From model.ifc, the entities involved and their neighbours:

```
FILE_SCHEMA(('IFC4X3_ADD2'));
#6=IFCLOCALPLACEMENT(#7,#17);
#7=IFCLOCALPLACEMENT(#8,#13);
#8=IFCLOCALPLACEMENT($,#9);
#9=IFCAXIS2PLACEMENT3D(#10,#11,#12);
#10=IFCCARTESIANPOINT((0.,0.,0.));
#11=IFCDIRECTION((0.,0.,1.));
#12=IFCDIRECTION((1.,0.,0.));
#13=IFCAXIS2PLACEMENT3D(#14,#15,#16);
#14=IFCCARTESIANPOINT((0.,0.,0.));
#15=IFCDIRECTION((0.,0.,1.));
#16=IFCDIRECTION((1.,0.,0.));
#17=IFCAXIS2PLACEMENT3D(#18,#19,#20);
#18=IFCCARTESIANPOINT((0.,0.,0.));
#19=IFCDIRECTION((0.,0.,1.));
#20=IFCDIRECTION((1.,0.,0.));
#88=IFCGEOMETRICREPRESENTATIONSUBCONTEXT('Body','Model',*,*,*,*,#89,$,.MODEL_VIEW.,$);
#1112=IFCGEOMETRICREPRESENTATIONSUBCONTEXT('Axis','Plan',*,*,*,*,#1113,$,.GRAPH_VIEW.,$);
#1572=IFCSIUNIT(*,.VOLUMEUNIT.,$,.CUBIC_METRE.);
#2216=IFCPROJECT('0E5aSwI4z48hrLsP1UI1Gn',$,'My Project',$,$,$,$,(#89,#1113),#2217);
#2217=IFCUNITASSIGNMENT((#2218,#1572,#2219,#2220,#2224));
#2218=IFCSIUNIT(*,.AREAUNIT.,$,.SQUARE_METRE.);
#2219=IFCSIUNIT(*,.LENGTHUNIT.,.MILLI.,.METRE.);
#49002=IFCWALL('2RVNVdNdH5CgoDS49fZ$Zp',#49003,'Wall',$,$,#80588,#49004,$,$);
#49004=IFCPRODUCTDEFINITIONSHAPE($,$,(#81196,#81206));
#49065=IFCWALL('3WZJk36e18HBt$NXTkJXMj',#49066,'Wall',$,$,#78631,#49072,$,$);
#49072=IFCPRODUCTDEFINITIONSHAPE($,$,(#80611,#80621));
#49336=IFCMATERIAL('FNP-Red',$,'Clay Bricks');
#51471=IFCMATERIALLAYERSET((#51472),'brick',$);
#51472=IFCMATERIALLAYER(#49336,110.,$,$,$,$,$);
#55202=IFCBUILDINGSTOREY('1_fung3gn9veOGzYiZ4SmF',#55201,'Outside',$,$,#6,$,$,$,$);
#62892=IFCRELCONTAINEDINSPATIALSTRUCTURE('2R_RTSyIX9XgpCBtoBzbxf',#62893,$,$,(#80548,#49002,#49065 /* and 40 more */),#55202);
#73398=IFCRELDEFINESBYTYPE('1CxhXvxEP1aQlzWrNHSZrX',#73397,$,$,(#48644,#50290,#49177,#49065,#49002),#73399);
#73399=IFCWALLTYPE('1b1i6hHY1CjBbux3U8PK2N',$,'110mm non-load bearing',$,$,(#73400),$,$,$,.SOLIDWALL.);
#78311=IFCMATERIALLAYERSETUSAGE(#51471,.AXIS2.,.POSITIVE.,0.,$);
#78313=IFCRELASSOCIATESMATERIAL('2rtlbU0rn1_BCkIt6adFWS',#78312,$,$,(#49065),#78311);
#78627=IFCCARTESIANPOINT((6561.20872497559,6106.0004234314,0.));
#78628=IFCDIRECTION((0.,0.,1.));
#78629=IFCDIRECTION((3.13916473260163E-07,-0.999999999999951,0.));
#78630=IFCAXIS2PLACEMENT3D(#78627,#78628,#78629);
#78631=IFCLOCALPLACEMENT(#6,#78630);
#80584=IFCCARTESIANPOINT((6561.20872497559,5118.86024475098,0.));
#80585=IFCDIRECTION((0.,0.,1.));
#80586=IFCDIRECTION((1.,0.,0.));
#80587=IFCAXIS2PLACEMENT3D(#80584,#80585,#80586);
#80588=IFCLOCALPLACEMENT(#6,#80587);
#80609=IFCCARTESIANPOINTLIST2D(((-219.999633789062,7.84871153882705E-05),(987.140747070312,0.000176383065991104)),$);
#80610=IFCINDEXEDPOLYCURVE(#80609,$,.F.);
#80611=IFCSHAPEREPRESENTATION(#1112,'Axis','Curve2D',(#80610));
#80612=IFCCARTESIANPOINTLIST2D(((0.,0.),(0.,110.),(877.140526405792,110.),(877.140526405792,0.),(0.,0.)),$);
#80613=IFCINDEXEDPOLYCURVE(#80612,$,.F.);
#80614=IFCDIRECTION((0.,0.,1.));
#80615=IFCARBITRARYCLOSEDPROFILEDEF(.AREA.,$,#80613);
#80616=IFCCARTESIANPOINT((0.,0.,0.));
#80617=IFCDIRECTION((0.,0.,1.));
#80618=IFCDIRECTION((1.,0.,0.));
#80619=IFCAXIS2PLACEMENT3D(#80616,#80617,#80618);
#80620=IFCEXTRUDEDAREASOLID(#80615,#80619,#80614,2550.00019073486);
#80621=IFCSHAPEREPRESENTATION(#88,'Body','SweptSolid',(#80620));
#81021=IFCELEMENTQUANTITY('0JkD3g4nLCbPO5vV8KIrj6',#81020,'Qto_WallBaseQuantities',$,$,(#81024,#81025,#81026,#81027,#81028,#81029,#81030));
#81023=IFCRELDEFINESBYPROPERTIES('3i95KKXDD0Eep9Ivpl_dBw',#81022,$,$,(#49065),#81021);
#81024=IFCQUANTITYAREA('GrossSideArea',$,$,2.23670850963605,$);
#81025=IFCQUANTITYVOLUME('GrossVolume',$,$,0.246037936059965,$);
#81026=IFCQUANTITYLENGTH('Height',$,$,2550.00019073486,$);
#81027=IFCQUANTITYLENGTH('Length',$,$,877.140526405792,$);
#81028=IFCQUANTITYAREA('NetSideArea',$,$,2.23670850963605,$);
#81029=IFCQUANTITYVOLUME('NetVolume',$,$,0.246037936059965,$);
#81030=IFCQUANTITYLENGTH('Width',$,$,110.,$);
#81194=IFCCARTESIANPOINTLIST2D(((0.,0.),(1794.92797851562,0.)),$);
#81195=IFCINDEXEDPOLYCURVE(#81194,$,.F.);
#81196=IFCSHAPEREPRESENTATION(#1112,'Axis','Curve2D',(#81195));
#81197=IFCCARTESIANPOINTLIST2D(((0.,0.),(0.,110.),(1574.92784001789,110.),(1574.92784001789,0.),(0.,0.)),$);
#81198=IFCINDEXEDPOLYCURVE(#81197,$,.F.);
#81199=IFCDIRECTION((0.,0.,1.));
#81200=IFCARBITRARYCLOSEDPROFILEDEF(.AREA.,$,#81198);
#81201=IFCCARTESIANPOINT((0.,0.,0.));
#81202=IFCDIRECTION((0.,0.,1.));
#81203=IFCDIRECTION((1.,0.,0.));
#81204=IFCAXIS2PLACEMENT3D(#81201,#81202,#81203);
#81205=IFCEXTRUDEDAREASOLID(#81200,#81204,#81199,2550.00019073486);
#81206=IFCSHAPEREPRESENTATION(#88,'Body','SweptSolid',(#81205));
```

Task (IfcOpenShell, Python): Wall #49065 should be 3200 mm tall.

```python
import ifcopenshell
import ifcopenshell.api.pset
import ifcopenshell.geom
import ifcopenshell.util.element
import ifcopenshell.util.representation
import ifcopenshell.util.shape
import ifcopenshell.util.unit

model = ifcopenshell.open("model.ifc")
unit_scale = ifcopenshell.util.unit.calculate_unit_scale(model)
area_scale = ifcopenshell.util.unit.calculate_unit_scale(model, "AREAUNIT")
volume_scale = ifcopenshell.util.unit.calculate_unit_scale(model, "VOLUMEUNIT")
settings = ifcopenshell.geom.settings()


def volume(element):
    """Net volume in cubic metres, openings subtracted."""
    shape = ifcopenshell.geom.create_shape(settings, element)
    return ifcopenshell.util.shape.get_volume(shape.geometry)


wall = model.by_guid("3WZJk36e18HBt$NXTkJXMj")
before = volume(wall)

body = ifcopenshell.util.representation.get_representation(wall, "Model", "Body")
solid = body.Items[0]
old_height = solid.Depth
solid.Depth = 3200.0
after = volume(wall)
thickness = 0.11  # wall thickness in metres

# Update the stored height, areas and volumes.
qto = model.by_id(ifcopenshell.util.element.get_pset(wall, "Qto_WallBaseQuantities", should_inherit=False)["id"])
ifcopenshell.api.pset.edit_qto(model, qto=qto, properties={
    "GrossSideArea": ifcopenshell.util.element.get_pset(wall, "Qto_WallBaseQuantities", "GrossSideArea") * solid.Depth / old_height,
    "GrossVolume": ifcopenshell.util.element.get_pset(wall, "Qto_WallBaseQuantities", "GrossVolume") * solid.Depth / old_height,
    "Height": solid.Depth,
    "NetSideArea": after / thickness / area_scale,
    "NetVolume": after / volume_scale,
})

print(f"height {old_height:g} -> {solid.Depth:g}, volume {before:.3f} -> {after:.3f} m3")

model.write("model_edited.ifc")
```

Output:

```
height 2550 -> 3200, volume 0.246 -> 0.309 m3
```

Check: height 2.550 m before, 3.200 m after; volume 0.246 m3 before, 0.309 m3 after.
